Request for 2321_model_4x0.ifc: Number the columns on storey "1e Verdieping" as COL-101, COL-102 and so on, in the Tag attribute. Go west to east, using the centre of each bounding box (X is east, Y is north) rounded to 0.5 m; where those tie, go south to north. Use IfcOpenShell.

First a look at what the model holds.

```python
import ifcopenshell
import ifcopenshell.util.element
import ifcopenshell.util.placement

model = ifcopenshell.open("2321_model_4x0.ifc")
print(model.schema)
storey = next(s for s in model.by_type("IfcBuildingStorey") if s.Name == "1e Verdieping")
columns = [e for e in ifcopenshell.util.element.get_decomposition(storey) if e.is_a("IfcColumn")]
for e in sorted(columns, key=lambda e: e.id()):
    origin = ifcopenshell.util.placement.get_local_placement(e.ObjectPlacement)[:3, 3]
    print(e.id(), e.Tag, e.Name, origin.round(2) + 0.0, sep=" | ")
```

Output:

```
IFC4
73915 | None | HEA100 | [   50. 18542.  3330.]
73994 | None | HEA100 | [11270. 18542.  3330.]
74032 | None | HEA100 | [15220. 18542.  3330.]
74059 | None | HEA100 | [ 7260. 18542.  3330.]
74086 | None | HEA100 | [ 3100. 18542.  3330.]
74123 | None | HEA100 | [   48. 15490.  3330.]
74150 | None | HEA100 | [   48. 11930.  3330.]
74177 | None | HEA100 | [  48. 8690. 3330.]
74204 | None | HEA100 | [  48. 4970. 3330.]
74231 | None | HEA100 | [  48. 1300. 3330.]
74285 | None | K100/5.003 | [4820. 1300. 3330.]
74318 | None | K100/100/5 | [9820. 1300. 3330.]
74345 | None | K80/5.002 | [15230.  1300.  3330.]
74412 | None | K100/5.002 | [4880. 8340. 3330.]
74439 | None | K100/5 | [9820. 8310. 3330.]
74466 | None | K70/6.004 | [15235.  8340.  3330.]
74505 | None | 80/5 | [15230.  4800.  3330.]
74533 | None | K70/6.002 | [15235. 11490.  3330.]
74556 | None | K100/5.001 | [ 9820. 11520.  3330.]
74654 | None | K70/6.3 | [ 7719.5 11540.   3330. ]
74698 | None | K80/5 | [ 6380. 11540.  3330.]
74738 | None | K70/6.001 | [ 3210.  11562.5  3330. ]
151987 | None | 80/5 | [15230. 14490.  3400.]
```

```python
import ifcopenshell
import ifcopenshell.geom
import ifcopenshell.util.element
import ifcopenshell.util.shape

model = ifcopenshell.open("2321_model_4x0.ifc")
settings = ifcopenshell.geom.settings()
settings.set("use-world-coords", True)


def centre(element):
    shape = ifcopenshell.geom.create_shape(settings, element)
    return ifcopenshell.util.shape.get_bbox_centroid(shape.geometry)


storey = next(s for s in model.by_type("IfcBuildingStorey") if s.Name == "1e Verdieping")
columns = [e for e in ifcopenshell.util.element.get_decomposition(storey) if e.is_a("IfcColumn")]

# Insertion points can sit at a corner or the storey origin, so sort by the geometry (in metres).
centres = {e: centre(e) for e in columns}
columns.sort(key=lambda e: (round(centres[e][0] / 0.5), centres[e][1]))

for i, e in enumerate(columns, start=1):
    number = f"COL-1{i:02d}"
    e.Tag = number
    print(e.id(), number)

model.write("2321_model_4x0_rev.ifc")
```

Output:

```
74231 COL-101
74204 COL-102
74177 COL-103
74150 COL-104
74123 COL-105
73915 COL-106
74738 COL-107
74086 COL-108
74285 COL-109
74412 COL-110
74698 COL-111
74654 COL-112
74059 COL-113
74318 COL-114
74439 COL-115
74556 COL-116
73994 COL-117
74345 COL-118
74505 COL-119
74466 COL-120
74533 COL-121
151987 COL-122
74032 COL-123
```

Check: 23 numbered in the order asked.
